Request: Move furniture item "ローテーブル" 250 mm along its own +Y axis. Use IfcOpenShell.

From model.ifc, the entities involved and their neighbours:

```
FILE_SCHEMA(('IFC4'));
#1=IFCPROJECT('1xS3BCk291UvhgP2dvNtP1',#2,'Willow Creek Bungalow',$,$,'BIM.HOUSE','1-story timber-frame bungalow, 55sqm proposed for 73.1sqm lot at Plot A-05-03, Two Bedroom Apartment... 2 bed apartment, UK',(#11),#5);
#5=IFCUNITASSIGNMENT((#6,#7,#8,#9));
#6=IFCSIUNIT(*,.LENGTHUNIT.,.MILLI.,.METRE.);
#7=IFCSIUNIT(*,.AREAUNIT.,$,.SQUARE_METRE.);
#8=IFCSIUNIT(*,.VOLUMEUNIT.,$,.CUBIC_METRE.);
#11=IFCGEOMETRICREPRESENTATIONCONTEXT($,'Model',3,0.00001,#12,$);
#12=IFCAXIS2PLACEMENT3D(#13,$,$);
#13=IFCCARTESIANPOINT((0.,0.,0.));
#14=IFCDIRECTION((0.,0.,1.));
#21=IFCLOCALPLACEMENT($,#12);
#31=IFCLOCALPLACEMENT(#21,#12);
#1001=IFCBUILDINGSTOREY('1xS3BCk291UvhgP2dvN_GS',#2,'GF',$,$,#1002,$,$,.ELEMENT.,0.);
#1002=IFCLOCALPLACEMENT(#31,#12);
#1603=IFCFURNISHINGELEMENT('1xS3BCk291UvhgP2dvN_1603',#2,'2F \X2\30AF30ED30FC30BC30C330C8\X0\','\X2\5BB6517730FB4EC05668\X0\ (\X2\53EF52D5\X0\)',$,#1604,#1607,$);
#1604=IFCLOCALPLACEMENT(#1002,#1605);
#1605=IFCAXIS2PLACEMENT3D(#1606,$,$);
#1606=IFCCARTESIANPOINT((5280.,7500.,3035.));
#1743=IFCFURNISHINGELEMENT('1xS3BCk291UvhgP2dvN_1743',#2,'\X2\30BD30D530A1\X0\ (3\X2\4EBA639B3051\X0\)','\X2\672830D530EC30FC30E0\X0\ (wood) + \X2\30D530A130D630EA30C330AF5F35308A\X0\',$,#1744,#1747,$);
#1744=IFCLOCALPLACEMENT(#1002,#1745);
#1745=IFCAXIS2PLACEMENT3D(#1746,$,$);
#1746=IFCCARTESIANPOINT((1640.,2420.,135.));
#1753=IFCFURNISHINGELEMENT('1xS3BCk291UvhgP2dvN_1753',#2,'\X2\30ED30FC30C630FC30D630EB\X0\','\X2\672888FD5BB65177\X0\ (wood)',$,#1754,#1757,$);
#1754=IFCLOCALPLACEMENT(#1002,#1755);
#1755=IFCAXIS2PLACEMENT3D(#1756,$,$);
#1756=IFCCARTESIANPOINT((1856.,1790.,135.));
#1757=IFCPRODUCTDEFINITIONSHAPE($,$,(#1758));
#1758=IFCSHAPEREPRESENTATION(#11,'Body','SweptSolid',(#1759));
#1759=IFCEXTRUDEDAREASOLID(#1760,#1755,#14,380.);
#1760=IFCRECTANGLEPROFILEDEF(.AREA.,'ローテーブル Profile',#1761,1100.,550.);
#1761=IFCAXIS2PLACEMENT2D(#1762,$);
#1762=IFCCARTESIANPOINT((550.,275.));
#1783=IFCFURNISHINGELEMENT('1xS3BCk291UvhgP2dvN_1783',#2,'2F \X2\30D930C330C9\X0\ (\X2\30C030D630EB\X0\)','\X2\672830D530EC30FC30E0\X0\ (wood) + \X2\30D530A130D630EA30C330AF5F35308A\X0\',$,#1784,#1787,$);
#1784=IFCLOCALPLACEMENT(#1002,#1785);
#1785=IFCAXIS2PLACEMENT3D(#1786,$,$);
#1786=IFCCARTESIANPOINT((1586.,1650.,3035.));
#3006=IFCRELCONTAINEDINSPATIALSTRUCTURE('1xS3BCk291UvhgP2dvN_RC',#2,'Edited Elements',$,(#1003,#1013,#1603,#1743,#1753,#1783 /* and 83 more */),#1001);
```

```python
import ifcopenshell
import ifcopenshell.api.geometry
import ifcopenshell.util.placement
import ifcopenshell.util.unit

model = ifcopenshell.open("model.ifc")
unit_scale = ifcopenshell.util.unit.calculate_unit_scale(model)

item = model.by_id(1753)
matrix = ifcopenshell.util.placement.get_local_placement(item.ObjectPlacement)
matrix[:3, 3] += matrix[:3, 1] * 0.25 / unit_scale
ifcopenshell.api.geometry.edit_object_placement(model, product=item, matrix=matrix, is_si=False)

print(ifcopenshell.util.placement.get_local_placement(item.ObjectPlacement).round(3) + 0.0)

model.write("model-out.ifc")
```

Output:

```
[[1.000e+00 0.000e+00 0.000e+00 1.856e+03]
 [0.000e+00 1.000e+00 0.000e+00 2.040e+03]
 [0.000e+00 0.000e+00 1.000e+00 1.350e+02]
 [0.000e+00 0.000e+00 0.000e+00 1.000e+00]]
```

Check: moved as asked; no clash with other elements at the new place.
